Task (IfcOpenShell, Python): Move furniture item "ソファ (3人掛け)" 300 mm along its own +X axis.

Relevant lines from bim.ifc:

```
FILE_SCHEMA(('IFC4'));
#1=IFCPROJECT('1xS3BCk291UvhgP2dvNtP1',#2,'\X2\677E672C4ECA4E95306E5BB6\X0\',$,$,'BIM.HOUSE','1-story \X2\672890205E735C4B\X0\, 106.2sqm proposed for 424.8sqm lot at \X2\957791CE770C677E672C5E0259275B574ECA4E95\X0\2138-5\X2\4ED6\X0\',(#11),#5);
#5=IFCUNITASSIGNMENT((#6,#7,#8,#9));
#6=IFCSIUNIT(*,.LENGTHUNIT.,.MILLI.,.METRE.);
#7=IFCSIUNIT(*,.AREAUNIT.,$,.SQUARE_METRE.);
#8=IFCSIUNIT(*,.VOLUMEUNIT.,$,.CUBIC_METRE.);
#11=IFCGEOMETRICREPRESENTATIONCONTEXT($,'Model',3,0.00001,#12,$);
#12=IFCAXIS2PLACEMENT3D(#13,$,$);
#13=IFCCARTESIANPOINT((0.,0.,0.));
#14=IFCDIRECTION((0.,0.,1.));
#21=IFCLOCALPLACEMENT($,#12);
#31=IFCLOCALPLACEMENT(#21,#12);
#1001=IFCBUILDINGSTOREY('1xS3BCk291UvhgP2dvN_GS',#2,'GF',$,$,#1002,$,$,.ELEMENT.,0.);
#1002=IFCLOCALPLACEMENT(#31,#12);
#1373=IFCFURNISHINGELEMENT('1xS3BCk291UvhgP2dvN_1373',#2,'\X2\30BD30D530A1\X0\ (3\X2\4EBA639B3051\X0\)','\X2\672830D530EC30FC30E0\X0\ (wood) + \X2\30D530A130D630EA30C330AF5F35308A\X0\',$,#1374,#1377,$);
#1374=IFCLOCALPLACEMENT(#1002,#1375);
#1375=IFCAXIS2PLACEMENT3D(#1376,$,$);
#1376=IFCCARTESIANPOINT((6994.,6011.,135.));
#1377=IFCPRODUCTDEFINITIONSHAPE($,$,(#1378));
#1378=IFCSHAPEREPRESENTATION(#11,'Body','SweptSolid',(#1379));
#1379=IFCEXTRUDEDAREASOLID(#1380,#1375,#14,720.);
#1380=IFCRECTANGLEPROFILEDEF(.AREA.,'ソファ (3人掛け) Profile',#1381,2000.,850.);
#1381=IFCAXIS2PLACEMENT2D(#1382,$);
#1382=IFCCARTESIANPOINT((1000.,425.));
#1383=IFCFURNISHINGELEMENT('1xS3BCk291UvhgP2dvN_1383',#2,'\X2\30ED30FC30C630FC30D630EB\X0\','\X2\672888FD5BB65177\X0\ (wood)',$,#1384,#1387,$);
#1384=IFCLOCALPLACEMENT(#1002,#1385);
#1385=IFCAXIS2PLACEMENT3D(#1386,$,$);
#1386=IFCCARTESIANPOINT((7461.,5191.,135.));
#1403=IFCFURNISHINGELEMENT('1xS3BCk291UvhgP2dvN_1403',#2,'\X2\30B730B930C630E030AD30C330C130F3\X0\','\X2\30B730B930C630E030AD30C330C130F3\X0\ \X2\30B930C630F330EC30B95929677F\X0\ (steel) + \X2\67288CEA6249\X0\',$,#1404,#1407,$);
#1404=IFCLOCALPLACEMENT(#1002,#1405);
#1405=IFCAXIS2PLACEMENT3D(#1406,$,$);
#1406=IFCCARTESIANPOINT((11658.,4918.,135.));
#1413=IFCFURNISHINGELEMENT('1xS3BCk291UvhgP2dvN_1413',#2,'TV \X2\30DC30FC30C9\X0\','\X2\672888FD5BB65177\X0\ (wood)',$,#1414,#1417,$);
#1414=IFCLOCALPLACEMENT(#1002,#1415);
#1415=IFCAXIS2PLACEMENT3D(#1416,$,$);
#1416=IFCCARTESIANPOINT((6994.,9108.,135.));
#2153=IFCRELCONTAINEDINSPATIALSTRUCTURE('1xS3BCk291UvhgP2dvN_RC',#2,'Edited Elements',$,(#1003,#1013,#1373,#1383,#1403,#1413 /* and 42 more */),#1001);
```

```python
import ifcopenshell
import ifcopenshell.api.geometry
import ifcopenshell.util.placement
import ifcopenshell.util.unit

model = ifcopenshell.open("bim.ifc")
unit_scale = ifcopenshell.util.unit.calculate_unit_scale(model)

item = model.by_id(1373)
matrix = ifcopenshell.util.placement.get_local_placement(item.ObjectPlacement)
matrix[:3, 3] += matrix[:3, 0] * 0.3 / unit_scale
ifcopenshell.api.geometry.edit_object_placement(model, product=item, matrix=matrix, is_si=False)

print(ifcopenshell.util.placement.get_local_placement(item.ObjectPlacement).round(3) + 0.0)

model.write("bim_v2.ifc")
```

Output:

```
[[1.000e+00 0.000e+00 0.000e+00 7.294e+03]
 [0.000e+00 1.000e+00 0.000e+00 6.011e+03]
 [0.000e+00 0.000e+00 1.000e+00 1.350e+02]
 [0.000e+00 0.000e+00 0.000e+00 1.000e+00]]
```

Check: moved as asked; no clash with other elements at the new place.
